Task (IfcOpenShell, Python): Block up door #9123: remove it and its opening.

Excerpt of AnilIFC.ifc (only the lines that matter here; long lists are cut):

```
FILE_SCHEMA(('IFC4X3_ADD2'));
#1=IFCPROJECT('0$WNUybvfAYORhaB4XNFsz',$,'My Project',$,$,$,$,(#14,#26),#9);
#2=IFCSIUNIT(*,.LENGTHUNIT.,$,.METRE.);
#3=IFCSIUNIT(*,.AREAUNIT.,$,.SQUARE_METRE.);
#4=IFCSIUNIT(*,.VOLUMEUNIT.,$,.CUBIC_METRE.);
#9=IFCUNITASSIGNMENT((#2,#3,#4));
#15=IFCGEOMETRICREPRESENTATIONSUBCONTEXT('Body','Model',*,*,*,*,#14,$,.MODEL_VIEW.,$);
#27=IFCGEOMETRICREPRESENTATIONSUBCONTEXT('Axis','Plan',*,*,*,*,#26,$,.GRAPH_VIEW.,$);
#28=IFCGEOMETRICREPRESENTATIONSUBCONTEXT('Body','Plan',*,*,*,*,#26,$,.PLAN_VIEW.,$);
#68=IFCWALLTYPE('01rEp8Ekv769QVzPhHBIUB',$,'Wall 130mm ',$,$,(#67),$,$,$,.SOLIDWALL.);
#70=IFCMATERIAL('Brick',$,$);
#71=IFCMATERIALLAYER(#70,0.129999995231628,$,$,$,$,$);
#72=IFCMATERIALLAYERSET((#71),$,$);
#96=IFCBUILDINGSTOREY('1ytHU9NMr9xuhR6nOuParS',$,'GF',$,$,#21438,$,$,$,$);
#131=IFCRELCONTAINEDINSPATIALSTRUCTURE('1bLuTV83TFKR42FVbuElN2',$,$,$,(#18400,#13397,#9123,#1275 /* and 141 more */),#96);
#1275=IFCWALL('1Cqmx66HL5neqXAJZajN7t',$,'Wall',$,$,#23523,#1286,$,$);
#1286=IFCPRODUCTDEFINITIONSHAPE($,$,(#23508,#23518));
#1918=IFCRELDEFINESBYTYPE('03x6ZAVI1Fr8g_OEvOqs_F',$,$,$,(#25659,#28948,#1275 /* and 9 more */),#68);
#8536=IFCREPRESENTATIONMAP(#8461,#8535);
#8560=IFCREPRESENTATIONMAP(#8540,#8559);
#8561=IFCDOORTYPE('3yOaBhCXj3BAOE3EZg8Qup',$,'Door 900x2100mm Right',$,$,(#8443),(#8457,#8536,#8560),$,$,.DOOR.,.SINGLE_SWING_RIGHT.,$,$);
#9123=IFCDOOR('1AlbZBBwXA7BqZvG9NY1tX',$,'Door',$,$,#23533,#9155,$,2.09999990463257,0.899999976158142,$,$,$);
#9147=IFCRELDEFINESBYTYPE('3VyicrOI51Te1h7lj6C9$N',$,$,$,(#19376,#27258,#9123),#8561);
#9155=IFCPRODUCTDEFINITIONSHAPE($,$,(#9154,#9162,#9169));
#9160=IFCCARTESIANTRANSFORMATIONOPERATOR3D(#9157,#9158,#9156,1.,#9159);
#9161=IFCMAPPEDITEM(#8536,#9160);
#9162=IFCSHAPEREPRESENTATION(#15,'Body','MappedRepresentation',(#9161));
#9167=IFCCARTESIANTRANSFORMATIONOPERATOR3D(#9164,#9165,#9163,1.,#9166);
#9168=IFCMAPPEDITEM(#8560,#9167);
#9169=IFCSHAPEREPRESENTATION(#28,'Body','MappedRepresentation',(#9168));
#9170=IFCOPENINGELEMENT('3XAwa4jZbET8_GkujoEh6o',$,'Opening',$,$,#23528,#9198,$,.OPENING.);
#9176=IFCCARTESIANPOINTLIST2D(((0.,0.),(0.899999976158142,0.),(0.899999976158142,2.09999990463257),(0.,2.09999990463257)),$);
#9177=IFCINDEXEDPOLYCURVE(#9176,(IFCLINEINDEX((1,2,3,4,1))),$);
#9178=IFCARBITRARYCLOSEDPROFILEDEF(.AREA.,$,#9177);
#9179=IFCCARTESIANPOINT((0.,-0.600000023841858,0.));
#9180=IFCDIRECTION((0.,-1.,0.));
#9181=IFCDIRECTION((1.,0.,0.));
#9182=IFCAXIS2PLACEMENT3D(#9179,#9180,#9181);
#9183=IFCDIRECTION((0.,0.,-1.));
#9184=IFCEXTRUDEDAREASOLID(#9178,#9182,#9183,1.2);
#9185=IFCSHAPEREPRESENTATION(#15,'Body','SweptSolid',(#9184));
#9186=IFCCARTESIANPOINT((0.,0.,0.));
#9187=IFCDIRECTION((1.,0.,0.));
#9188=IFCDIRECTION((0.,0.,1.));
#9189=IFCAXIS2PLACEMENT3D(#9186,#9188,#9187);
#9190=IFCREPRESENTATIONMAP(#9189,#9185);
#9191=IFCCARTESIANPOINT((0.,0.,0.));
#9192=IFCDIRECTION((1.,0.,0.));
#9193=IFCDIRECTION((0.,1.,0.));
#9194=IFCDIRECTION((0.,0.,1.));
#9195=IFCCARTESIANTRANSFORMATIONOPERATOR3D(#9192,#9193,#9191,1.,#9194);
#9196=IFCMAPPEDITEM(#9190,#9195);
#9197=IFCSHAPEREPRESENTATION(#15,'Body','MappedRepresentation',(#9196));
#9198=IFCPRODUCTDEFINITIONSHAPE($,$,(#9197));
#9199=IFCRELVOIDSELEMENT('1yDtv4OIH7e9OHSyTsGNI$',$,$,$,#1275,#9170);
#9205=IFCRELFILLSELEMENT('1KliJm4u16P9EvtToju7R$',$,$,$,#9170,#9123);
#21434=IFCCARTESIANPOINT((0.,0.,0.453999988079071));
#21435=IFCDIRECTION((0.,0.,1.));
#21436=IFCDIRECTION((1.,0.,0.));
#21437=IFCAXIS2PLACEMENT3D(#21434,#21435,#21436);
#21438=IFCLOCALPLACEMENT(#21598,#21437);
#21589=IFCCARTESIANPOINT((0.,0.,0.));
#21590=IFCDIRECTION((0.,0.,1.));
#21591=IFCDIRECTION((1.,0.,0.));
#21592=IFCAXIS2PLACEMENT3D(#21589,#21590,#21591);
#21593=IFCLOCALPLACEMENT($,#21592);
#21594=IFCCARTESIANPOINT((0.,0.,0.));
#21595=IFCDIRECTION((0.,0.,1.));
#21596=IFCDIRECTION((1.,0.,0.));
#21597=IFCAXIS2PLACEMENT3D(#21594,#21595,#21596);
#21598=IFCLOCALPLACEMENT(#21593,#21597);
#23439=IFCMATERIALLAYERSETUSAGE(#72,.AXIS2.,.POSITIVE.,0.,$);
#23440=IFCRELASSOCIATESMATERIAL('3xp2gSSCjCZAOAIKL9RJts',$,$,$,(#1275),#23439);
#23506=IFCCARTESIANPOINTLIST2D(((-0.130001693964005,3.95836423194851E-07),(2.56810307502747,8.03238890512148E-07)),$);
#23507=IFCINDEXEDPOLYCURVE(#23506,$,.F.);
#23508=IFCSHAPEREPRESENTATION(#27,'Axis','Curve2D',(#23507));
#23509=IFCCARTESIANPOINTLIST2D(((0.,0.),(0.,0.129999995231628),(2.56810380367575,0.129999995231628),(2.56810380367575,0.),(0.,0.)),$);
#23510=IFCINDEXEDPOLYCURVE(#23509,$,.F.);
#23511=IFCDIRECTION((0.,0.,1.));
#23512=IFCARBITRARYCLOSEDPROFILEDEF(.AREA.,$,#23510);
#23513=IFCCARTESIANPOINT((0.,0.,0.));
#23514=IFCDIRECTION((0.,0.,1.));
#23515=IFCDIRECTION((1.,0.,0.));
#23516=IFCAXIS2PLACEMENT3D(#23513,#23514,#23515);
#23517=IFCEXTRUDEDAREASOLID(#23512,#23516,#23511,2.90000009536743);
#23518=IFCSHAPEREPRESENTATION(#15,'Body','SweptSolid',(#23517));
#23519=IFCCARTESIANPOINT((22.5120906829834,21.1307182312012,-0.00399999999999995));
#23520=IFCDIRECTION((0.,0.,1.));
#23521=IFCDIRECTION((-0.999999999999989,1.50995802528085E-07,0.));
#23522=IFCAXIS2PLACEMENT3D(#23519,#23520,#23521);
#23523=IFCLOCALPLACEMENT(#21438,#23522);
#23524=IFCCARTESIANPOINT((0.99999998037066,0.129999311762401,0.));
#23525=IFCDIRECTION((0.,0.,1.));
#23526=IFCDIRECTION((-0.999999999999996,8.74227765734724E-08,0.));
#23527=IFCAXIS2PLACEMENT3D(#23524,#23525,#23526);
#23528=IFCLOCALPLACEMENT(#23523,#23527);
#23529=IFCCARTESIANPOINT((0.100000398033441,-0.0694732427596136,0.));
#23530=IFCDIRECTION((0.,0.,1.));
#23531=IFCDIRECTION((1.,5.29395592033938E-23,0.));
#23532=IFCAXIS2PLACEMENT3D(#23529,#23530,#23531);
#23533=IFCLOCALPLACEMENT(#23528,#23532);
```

```python
import ifcopenshell
import ifcopenshell.api.feature
import ifcopenshell.api.root
import ifcopenshell.geom
import ifcopenshell.util.shape

model = ifcopenshell.open("AnilIFC.ifc")
settings = ifcopenshell.geom.settings()


def volume(element):
    """Net volume in cubic metres, openings subtracted."""
    shape = ifcopenshell.geom.create_shape(settings, element)
    return ifcopenshell.util.shape.get_volume(shape.geometry)


door = model.by_guid("1AlbZBBwXA7BqZvG9NY1tX")
opening = door.FillsVoids[0].RelatingOpeningElement
wall = opening.VoidsElements[0].RelatingBuildingElement
before = volume(wall)

ifcopenshell.api.root.remove_product(model, product=door)
ifcopenshell.api.feature.remove_feature(model, feature=opening)

after = volume(wall)

print(f"wall volume {before:.3f} -> {after:.3f} m3")

model.write("AnilIFC_v2.ifc")
```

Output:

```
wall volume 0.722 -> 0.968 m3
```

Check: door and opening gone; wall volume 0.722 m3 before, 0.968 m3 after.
